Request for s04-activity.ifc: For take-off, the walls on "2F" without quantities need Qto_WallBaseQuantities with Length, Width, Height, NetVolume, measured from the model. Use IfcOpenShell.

First a look at what the model holds.

```python
import ifcopenshell
import ifcopenshell.util.element
import ifcopenshell.util.unit

model = ifcopenshell.open("s04-activity.ifc")
print(model.schema)
for unit_type in ("LENGTHUNIT", "AREAUNIT", "VOLUMEUNIT"):
    print(unit_type, ifcopenshell.util.unit.calculate_unit_scale(model, unit_type))
storey = next(s for s in model.by_type("IfcBuildingStorey") if s.Name == "2F")
walls = [e for e in ifcopenshell.util.element.get_decomposition(storey) if e.is_a("IfcWall")]
for e in sorted(walls, key=lambda e: e.id()):
    print(e.id(), e.is_a(), e.Name, list(ifcopenshell.util.element.get_psets(e, qtos_only=True)), sep=" | ")
```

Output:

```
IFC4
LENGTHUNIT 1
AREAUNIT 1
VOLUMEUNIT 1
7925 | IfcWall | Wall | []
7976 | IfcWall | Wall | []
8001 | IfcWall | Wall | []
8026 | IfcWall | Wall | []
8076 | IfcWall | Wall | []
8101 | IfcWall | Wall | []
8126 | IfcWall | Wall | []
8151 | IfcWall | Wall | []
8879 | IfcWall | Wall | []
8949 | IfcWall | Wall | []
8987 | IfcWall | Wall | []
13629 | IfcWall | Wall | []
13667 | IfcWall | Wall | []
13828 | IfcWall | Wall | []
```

```python
import ifcopenshell
import ifcopenshell.api.pset
import ifcopenshell.geom
import ifcopenshell.util.element
import ifcopenshell.util.shape
import ifcopenshell.util.unit

model = ifcopenshell.open("s04-activity.ifc")
unit_scale = ifcopenshell.util.unit.calculate_unit_scale(model)
volume_scale = ifcopenshell.util.unit.calculate_unit_scale(model, "VOLUMEUNIT")
settings = ifcopenshell.geom.settings()

storey = next(s for s in model.by_type("IfcBuildingStorey") if s.Name == "2F")
walls = [e for e in ifcopenshell.util.element.get_decomposition(storey) if e.is_a("IfcWall")]

for e in sorted(walls, key=lambda e: e.id()):
    if ifcopenshell.util.element.get_psets(e, qtos_only=True, should_inherit=False):
        continue
    # Geometry comes back in metres, in the element's own axes.
    shape = ifcopenshell.geom.create_shape(settings, e)
    values = {
        "Length": ifcopenshell.util.shape.get_x(shape.geometry) / unit_scale,
        "Width": ifcopenshell.util.shape.get_y(shape.geometry) / unit_scale,
        "Height": ifcopenshell.util.shape.get_z(shape.geometry) / unit_scale,
        "NetVolume": ifcopenshell.util.shape.get_volume(shape.geometry) / volume_scale,
    }
    qto = ifcopenshell.api.pset.add_qto(model, product=e, name="Qto_WallBaseQuantities")
    ifcopenshell.api.pset.edit_qto(model, qto=qto, properties=values)
    print(e.id(), {k: round(v, 3) for k, v in values.items()})

model.write("s04-activity_updated.ifc")
```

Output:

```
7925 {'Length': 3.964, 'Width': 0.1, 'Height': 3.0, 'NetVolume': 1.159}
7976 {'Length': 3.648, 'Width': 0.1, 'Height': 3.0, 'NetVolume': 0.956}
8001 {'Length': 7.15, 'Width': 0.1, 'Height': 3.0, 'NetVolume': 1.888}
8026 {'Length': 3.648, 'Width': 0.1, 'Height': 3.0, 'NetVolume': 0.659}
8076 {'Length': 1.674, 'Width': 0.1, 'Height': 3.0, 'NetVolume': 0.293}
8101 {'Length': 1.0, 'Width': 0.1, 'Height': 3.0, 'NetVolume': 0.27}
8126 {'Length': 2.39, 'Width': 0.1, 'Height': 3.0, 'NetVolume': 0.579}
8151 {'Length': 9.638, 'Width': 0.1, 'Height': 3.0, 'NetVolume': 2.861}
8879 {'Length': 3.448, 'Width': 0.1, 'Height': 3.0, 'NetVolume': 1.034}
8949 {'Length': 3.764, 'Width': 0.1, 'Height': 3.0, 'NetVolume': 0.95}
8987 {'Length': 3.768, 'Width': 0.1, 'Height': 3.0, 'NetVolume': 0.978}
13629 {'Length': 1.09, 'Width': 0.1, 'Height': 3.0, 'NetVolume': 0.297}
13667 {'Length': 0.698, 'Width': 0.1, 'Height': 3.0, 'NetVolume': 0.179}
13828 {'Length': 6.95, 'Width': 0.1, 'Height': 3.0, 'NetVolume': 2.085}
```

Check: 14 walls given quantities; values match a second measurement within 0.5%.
